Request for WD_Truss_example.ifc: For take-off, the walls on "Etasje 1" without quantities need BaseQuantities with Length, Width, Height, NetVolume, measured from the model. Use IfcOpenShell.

First a look at what the model holds.

```python
import ifcopenshell
import ifcopenshell.util.element
import ifcopenshell.util.unit

model = ifcopenshell.open("WD_Truss_example.ifc")
print(model.schema)
for unit_type in ("LENGTHUNIT", "AREAUNIT", "VOLUMEUNIT"):
    print(unit_type, ifcopenshell.util.unit.calculate_unit_scale(model, unit_type))
storey = next(s for s in model.by_type("IfcBuildingStorey") if s.Name == "Etasje 1")
walls = [e for e in ifcopenshell.util.element.get_decomposition(storey) if e.is_a("IfcWall")]
for e in sorted(walls, key=lambda e: e.id()):
    print(e.id(), e.is_a(), e.Name, list(ifcopenshell.util.element.get_psets(e, qtos_only=True)), sep=" | ")
```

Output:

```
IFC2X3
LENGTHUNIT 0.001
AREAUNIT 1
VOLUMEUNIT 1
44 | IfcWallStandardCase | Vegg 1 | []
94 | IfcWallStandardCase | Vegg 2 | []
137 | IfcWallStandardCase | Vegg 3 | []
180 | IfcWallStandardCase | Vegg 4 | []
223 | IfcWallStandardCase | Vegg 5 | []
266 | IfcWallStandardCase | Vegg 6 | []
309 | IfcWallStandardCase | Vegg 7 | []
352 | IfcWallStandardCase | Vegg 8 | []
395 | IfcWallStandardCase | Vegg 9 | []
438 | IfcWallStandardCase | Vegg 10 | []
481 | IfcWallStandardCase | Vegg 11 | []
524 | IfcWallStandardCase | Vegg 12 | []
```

```python
import ifcopenshell
import ifcopenshell.api.pset
import ifcopenshell.geom
import ifcopenshell.util.element
import ifcopenshell.util.shape
import ifcopenshell.util.unit

model = ifcopenshell.open("WD_Truss_example.ifc")
unit_scale = ifcopenshell.util.unit.calculate_unit_scale(model)
volume_scale = ifcopenshell.util.unit.calculate_unit_scale(model, "VOLUMEUNIT")
settings = ifcopenshell.geom.settings()

storey = next(s for s in model.by_type("IfcBuildingStorey") if s.Name == "Etasje 1")
walls = [e for e in ifcopenshell.util.element.get_decomposition(storey) if e.is_a("IfcWall")]

for e in sorted(walls, key=lambda e: e.id()):
    if ifcopenshell.util.element.get_psets(e, qtos_only=True, should_inherit=False):
        continue
    # Geometry comes back in metres, in the element's own axes.
    shape = ifcopenshell.geom.create_shape(settings, e)
    values = {
        "Length": ifcopenshell.util.shape.get_x(shape.geometry) / unit_scale,
        "Width": ifcopenshell.util.shape.get_y(shape.geometry) / unit_scale,
        "Height": ifcopenshell.util.shape.get_z(shape.geometry) / unit_scale,
        "NetVolume": ifcopenshell.util.shape.get_volume(shape.geometry) / volume_scale,
    }
    qto = ifcopenshell.api.pset.add_qto(model, product=e, name="BaseQuantities")
    ifcopenshell.api.pset.edit_qto(model, qto=qto, properties=values)
    print(e.id(), {k: round(v, 3) for k, v in values.items()})

model.write("WD_Truss_example_edited.ifc")
```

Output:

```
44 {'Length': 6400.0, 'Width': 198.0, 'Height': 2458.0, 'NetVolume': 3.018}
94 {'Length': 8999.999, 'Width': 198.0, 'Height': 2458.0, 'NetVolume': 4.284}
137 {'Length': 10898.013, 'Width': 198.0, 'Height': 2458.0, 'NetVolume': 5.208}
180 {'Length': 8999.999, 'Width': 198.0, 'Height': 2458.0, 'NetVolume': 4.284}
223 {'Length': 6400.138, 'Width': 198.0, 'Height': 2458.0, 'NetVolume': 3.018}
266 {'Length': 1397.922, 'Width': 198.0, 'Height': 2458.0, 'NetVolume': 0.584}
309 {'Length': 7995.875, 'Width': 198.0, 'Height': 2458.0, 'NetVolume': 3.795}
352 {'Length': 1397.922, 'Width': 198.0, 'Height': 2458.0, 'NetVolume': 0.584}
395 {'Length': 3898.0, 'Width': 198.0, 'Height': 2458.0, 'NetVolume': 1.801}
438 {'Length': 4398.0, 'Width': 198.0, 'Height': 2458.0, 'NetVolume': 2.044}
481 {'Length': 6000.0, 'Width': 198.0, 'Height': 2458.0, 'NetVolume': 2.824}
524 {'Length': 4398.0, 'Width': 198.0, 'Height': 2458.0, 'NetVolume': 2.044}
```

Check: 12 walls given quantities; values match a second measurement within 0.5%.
